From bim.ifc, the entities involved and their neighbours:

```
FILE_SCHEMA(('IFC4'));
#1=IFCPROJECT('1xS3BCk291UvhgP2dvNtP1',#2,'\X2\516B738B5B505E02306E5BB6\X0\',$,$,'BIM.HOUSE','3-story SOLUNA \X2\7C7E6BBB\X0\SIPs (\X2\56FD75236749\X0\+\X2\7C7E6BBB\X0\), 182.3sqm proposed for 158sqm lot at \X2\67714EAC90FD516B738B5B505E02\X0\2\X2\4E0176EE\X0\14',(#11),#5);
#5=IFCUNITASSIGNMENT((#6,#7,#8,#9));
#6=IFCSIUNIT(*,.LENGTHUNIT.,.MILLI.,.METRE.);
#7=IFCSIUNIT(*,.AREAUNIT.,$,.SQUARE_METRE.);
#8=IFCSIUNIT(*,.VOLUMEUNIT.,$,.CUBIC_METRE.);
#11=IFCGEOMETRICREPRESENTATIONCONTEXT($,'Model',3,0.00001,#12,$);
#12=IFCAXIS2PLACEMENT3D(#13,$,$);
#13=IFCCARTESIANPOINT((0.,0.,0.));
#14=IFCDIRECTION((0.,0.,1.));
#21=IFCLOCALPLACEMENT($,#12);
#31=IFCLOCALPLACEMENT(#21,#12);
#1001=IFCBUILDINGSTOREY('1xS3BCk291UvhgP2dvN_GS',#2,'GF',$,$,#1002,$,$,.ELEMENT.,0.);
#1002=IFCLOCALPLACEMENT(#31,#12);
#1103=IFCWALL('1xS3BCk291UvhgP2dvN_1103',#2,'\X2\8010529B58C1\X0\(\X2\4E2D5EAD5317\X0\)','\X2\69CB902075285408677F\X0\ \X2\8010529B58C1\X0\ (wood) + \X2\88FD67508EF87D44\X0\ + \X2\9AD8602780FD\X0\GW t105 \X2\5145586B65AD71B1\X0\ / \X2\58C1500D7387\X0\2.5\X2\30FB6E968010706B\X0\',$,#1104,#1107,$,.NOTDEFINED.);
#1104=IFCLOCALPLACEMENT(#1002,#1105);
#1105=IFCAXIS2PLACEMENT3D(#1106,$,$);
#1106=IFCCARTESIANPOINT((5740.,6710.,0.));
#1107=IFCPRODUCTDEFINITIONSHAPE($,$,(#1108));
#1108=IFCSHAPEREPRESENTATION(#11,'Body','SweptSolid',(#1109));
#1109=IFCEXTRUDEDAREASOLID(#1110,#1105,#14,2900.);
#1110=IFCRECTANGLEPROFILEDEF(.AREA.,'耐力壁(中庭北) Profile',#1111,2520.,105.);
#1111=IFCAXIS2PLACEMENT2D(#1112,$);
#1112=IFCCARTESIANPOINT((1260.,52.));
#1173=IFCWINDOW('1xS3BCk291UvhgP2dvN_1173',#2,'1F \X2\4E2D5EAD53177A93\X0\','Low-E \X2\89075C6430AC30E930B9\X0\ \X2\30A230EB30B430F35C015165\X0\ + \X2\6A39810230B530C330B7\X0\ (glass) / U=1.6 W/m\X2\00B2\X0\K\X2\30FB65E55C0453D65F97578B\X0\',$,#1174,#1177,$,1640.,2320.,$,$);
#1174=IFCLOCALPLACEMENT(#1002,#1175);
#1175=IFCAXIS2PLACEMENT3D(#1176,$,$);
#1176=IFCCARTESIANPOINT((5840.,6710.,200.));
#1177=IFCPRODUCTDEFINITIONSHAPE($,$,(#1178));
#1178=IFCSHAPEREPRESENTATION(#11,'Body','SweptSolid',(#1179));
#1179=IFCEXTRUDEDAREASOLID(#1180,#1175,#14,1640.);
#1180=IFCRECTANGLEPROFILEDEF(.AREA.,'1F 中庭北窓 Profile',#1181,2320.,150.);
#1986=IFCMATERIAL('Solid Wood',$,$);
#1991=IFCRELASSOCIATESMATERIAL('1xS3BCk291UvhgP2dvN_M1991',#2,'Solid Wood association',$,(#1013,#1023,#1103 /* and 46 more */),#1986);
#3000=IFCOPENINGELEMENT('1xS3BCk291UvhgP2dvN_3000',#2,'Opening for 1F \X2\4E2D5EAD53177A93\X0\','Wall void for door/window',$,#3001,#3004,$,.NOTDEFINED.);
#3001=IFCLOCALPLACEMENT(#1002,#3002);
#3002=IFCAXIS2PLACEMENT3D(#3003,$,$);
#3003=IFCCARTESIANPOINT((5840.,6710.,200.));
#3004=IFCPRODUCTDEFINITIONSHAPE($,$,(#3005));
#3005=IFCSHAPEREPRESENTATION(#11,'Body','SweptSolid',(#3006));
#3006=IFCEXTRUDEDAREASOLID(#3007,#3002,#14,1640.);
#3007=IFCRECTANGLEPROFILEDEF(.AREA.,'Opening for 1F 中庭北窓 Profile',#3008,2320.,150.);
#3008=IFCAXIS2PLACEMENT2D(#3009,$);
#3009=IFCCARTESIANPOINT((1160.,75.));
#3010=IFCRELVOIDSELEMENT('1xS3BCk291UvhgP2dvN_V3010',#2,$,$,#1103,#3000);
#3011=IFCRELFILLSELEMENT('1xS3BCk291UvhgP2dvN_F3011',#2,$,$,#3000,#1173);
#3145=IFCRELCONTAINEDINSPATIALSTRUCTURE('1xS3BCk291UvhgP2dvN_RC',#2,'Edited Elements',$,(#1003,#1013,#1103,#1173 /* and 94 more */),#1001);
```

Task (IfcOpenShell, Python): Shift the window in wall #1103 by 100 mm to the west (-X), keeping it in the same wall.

```python
import ifcopenshell
import ifcopenshell.api.geometry
import ifcopenshell.util.placement
import ifcopenshell.util.unit

model = ifcopenshell.open("bim.ifc")
unit_scale = ifcopenshell.util.unit.calculate_unit_scale(model)

window = model.by_guid("1xS3BCk291UvhgP2dvN_1173")
opening = window.FillsVoids[0].RelatingOpeningElement
wall = opening.VoidsElements[0].RelatingBuildingElement

wall_matrix = ifcopenshell.util.placement.get_local_placement(wall.ObjectPlacement)
shift = wall_matrix[:3, 0] * -0.1 / unit_scale
before = ifcopenshell.util.placement.get_local_placement(window.ObjectPlacement)[:3, 3].copy()

# The window is not placed relative to its opening, so move both.
for product in (opening, window):
    matrix = ifcopenshell.util.placement.get_local_placement(product.ObjectPlacement)
    matrix[:3, 3] += shift
    ifcopenshell.api.geometry.edit_object_placement(model, product=product, matrix=matrix, is_si=False)

after = ifcopenshell.util.placement.get_local_placement(window.ObjectPlacement)[:3, 3]
print("window moved by", (after - before).round(3) + 0.0)

model.write("bim_v2.ifc")
```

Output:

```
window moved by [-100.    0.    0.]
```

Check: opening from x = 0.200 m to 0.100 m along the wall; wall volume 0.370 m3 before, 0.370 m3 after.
